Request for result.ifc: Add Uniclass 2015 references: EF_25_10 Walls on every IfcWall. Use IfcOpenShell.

First a look at what the model holds.

```python
import ifcopenshell

model = ifcopenshell.open("result.ifc")
print(model.schema)
print("classifications:", [c.Name for c in model.by_type("IfcClassification")])
for ifc_class in ("IfcDoor", "IfcRoof", "IfcStair", "IfcWall", "IfcWindow"):
    print(ifc_class, len(model.by_type(ifc_class)))
```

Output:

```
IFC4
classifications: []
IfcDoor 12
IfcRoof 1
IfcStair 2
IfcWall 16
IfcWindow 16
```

```python
import ifcopenshell
import ifcopenshell.api.classification

model = ifcopenshell.open("result.ifc")

system = ifcopenshell.api.classification.add_classification(model, classification="Uniclass 2015")

codes = {
    "IfcWall": ("EF_25_10", "Walls"),
}
for ifc_class, (code, name) in codes.items():
    products = model.by_type(ifc_class)
    ifcopenshell.api.classification.add_reference(
        model, products=products, classification=system, identification=code, name=name
    )
    print(code, len(products))

model.write("result_rev.ifc")
```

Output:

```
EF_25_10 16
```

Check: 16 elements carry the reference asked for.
